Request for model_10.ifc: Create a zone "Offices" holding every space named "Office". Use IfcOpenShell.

First a look at what the model holds.

```python
import ifcopenshell

model = ifcopenshell.open("model_10.ifc")
print(model.schema)
seen = {}
for space in model.by_type("IfcSpace"):
    seen[space.LongName] = seen.get(space.LongName, 0) + 1
for name, count in sorted(seen.items(), key=str):
    print(count, "x", name)
print("zones:", [z.Name for z in model.by_type("IfcZone")][:20])
```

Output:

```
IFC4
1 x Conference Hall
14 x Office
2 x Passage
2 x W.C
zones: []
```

```python
import ifcopenshell
import ifcopenshell.api.group
import ifcopenshell.api.root

model = ifcopenshell.open("model_10.ifc")

names = {"Office"}
spaces = [s for s in model.by_type("IfcSpace") if s.LongName in names]

zone = ifcopenshell.api.root.create_entity(model, ifc_class="IfcZone", name="Offices")
ifcopenshell.api.group.assign_group(model, products=spaces, group=zone)
print(len(spaces), "spaces in", zone.Name)

model.write("model_10_updated.ifc")
```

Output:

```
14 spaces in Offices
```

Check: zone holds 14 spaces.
